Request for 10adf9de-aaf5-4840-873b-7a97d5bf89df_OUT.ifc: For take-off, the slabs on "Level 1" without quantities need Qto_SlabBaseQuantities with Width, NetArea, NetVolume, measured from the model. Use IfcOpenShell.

First a look at what the model holds.

```python
import ifcopenshell
import ifcopenshell.util.element
import ifcopenshell.util.unit

model = ifcopenshell.open("10adf9de-aaf5-4840-873b-7a97d5bf89df_OUT.ifc")
print(model.schema)
for unit_type in ("LENGTHUNIT", "AREAUNIT", "VOLUMEUNIT"):
    print(unit_type, ifcopenshell.util.unit.calculate_unit_scale(model, unit_type))
storey = next(s for s in model.by_type("IfcBuildingStorey") if s.Name == "Level 1")
slabs = [e for e in ifcopenshell.util.element.get_decomposition(storey) if e.is_a("IfcSlab")]
for e in sorted(slabs, key=lambda e: e.id()):
    print(e.id(), e.is_a(), e.Name, list(ifcopenshell.util.element.get_psets(e, qtos_only=True)), sep=" | ")
```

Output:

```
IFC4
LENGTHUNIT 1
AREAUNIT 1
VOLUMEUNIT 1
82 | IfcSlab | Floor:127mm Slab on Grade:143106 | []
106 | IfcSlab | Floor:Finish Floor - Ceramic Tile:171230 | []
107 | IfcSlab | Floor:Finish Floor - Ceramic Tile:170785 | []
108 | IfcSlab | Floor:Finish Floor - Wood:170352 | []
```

```python
import ifcopenshell
import ifcopenshell.api.pset
import ifcopenshell.geom
import ifcopenshell.util.element
import ifcopenshell.util.shape
import ifcopenshell.util.unit

model = ifcopenshell.open("10adf9de-aaf5-4840-873b-7a97d5bf89df_OUT.ifc")
unit_scale = ifcopenshell.util.unit.calculate_unit_scale(model)
area_scale = ifcopenshell.util.unit.calculate_unit_scale(model, "AREAUNIT")
volume_scale = ifcopenshell.util.unit.calculate_unit_scale(model, "VOLUMEUNIT")
settings = ifcopenshell.geom.settings()

storey = next(s for s in model.by_type("IfcBuildingStorey") if s.Name == "Level 1")
slabs = [e for e in ifcopenshell.util.element.get_decomposition(storey) if e.is_a("IfcSlab")]

for e in sorted(slabs, key=lambda e: e.id()):
    if ifcopenshell.util.element.get_psets(e, qtos_only=True, should_inherit=False):
        continue
    # Geometry comes back in metres, in the element's own axes.
    shape = ifcopenshell.geom.create_shape(settings, e)
    values = {
        "Width": ifcopenshell.util.shape.get_z(shape.geometry) / unit_scale,
        "NetArea": ifcopenshell.util.shape.get_footprint_area(shape.geometry) / area_scale,
        "NetVolume": ifcopenshell.util.shape.get_volume(shape.geometry) / volume_scale,
    }
    qto = ifcopenshell.api.pset.add_qto(model, product=e, name="Qto_SlabBaseQuantities")
    ifcopenshell.api.pset.edit_qto(model, qto=qto, properties=values)
    print(e.id(), {k: round(v, 3) for k, v in values.items()})

model.write("10adf9de-aaf5-4840-873b-7a97d5bf89df_OUT-out.ifc")
```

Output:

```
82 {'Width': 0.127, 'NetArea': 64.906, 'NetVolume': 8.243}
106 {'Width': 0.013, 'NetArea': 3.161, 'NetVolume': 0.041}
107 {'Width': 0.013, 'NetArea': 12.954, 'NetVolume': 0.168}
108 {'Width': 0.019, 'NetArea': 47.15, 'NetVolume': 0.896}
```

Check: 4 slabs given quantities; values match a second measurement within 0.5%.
